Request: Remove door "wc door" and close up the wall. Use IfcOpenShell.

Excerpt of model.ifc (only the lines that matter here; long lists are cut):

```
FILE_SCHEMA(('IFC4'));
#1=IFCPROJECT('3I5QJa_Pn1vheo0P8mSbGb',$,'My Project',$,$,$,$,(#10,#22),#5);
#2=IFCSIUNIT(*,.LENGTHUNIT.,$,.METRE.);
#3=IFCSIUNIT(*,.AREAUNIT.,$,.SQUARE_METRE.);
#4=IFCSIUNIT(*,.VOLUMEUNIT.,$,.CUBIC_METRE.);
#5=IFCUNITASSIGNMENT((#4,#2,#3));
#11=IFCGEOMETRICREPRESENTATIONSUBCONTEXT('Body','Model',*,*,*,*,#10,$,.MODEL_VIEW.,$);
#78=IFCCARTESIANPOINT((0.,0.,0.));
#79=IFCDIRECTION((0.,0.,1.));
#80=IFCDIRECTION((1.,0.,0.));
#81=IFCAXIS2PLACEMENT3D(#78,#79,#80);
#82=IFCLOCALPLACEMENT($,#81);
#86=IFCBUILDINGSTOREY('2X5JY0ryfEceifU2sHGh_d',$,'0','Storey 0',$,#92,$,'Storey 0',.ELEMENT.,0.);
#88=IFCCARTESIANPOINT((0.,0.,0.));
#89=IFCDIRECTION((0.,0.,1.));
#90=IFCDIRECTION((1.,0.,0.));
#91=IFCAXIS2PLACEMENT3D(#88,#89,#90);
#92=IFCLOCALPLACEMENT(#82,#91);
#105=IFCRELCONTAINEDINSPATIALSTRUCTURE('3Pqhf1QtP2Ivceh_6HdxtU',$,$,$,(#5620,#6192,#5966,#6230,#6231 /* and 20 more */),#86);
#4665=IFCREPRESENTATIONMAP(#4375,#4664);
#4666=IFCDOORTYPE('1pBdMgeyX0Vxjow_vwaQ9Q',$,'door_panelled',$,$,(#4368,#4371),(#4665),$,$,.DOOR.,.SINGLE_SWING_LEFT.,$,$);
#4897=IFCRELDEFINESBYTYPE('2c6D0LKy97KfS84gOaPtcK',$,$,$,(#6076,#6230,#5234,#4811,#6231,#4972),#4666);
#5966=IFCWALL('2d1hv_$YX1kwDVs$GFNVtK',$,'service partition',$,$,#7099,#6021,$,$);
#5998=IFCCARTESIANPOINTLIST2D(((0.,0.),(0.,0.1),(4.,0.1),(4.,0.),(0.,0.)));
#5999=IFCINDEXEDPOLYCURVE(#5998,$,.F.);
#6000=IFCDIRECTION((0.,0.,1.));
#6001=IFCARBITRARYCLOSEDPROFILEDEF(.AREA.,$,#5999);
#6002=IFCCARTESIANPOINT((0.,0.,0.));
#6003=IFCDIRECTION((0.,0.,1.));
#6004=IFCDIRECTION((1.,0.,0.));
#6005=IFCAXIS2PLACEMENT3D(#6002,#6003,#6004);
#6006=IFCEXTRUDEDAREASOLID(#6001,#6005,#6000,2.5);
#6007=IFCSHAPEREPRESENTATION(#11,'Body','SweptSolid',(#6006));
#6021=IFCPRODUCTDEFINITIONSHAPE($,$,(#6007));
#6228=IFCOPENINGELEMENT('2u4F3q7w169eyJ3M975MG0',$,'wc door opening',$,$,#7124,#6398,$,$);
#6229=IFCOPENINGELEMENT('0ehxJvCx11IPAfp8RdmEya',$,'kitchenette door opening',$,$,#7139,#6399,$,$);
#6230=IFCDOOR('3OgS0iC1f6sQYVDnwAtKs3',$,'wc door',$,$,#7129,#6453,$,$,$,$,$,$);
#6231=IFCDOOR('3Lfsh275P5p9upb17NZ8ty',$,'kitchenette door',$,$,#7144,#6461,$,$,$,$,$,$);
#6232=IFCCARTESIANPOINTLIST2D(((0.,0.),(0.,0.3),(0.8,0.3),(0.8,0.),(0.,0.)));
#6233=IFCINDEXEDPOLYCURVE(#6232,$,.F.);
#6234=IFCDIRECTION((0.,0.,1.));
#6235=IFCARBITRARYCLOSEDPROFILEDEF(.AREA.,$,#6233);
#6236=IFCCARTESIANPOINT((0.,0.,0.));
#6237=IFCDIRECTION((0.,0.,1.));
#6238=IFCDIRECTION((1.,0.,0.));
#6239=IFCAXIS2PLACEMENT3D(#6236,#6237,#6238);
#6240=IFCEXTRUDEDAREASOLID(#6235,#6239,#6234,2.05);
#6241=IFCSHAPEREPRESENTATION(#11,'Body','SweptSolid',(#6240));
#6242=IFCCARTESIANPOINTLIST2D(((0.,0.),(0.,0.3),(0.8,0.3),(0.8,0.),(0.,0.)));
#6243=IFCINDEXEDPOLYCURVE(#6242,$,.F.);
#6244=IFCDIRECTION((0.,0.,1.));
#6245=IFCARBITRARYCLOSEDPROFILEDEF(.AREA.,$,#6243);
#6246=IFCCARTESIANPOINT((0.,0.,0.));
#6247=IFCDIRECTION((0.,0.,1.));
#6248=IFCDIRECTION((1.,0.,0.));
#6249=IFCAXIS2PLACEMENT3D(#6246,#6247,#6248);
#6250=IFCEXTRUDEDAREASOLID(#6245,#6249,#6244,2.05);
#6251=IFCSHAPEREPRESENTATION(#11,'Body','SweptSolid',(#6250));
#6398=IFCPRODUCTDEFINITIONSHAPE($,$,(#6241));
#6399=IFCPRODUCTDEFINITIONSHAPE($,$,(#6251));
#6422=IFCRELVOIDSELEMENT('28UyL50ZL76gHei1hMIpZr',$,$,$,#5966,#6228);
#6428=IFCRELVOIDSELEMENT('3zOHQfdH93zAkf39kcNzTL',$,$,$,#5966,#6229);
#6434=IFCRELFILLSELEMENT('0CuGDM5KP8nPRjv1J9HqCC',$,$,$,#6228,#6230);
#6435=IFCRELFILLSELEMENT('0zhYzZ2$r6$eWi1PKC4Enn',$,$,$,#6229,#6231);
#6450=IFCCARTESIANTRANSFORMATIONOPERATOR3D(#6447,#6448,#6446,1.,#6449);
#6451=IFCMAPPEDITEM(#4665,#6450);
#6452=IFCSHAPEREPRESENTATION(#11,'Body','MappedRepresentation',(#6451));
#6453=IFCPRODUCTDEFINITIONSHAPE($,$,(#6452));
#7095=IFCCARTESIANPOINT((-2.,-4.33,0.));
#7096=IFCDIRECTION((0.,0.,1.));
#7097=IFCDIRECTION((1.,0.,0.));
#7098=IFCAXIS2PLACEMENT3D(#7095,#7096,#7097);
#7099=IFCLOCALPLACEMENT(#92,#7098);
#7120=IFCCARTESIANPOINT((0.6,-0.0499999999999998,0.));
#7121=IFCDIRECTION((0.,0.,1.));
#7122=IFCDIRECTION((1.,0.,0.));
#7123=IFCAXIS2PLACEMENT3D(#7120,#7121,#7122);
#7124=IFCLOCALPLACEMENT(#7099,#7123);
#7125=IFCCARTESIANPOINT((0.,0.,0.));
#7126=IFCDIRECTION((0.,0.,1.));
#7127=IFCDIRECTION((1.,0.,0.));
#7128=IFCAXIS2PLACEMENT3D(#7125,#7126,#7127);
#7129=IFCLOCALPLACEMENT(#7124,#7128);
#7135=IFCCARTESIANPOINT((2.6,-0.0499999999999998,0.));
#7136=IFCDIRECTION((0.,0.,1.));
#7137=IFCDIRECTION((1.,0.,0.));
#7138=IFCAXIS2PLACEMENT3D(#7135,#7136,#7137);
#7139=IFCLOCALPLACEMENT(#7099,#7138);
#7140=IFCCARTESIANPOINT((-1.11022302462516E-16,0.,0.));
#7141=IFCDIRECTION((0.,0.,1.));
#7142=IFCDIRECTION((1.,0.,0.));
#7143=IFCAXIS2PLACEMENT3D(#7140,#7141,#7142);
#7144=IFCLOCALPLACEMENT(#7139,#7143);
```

```python
import ifcopenshell
import ifcopenshell.api.feature
import ifcopenshell.api.root
import ifcopenshell.geom
import ifcopenshell.util.shape

model = ifcopenshell.open("model.ifc")
settings = ifcopenshell.geom.settings()


def volume(element):
    """Net volume in cubic metres, openings subtracted."""
    shape = ifcopenshell.geom.create_shape(settings, element)
    return ifcopenshell.util.shape.get_volume(shape.geometry)


door = model.by_id(6230)
opening = door.FillsVoids[0].RelatingOpeningElement
wall = opening.VoidsElements[0].RelatingBuildingElement
before = volume(wall)

ifcopenshell.api.root.remove_product(model, product=door)
ifcopenshell.api.feature.remove_feature(model, feature=opening)

after = volume(wall)

print(f"wall volume {before:.3f} -> {after:.3f} m3")

model.write("model-out.ifc")
```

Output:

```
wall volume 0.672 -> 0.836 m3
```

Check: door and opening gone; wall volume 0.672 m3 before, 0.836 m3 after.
